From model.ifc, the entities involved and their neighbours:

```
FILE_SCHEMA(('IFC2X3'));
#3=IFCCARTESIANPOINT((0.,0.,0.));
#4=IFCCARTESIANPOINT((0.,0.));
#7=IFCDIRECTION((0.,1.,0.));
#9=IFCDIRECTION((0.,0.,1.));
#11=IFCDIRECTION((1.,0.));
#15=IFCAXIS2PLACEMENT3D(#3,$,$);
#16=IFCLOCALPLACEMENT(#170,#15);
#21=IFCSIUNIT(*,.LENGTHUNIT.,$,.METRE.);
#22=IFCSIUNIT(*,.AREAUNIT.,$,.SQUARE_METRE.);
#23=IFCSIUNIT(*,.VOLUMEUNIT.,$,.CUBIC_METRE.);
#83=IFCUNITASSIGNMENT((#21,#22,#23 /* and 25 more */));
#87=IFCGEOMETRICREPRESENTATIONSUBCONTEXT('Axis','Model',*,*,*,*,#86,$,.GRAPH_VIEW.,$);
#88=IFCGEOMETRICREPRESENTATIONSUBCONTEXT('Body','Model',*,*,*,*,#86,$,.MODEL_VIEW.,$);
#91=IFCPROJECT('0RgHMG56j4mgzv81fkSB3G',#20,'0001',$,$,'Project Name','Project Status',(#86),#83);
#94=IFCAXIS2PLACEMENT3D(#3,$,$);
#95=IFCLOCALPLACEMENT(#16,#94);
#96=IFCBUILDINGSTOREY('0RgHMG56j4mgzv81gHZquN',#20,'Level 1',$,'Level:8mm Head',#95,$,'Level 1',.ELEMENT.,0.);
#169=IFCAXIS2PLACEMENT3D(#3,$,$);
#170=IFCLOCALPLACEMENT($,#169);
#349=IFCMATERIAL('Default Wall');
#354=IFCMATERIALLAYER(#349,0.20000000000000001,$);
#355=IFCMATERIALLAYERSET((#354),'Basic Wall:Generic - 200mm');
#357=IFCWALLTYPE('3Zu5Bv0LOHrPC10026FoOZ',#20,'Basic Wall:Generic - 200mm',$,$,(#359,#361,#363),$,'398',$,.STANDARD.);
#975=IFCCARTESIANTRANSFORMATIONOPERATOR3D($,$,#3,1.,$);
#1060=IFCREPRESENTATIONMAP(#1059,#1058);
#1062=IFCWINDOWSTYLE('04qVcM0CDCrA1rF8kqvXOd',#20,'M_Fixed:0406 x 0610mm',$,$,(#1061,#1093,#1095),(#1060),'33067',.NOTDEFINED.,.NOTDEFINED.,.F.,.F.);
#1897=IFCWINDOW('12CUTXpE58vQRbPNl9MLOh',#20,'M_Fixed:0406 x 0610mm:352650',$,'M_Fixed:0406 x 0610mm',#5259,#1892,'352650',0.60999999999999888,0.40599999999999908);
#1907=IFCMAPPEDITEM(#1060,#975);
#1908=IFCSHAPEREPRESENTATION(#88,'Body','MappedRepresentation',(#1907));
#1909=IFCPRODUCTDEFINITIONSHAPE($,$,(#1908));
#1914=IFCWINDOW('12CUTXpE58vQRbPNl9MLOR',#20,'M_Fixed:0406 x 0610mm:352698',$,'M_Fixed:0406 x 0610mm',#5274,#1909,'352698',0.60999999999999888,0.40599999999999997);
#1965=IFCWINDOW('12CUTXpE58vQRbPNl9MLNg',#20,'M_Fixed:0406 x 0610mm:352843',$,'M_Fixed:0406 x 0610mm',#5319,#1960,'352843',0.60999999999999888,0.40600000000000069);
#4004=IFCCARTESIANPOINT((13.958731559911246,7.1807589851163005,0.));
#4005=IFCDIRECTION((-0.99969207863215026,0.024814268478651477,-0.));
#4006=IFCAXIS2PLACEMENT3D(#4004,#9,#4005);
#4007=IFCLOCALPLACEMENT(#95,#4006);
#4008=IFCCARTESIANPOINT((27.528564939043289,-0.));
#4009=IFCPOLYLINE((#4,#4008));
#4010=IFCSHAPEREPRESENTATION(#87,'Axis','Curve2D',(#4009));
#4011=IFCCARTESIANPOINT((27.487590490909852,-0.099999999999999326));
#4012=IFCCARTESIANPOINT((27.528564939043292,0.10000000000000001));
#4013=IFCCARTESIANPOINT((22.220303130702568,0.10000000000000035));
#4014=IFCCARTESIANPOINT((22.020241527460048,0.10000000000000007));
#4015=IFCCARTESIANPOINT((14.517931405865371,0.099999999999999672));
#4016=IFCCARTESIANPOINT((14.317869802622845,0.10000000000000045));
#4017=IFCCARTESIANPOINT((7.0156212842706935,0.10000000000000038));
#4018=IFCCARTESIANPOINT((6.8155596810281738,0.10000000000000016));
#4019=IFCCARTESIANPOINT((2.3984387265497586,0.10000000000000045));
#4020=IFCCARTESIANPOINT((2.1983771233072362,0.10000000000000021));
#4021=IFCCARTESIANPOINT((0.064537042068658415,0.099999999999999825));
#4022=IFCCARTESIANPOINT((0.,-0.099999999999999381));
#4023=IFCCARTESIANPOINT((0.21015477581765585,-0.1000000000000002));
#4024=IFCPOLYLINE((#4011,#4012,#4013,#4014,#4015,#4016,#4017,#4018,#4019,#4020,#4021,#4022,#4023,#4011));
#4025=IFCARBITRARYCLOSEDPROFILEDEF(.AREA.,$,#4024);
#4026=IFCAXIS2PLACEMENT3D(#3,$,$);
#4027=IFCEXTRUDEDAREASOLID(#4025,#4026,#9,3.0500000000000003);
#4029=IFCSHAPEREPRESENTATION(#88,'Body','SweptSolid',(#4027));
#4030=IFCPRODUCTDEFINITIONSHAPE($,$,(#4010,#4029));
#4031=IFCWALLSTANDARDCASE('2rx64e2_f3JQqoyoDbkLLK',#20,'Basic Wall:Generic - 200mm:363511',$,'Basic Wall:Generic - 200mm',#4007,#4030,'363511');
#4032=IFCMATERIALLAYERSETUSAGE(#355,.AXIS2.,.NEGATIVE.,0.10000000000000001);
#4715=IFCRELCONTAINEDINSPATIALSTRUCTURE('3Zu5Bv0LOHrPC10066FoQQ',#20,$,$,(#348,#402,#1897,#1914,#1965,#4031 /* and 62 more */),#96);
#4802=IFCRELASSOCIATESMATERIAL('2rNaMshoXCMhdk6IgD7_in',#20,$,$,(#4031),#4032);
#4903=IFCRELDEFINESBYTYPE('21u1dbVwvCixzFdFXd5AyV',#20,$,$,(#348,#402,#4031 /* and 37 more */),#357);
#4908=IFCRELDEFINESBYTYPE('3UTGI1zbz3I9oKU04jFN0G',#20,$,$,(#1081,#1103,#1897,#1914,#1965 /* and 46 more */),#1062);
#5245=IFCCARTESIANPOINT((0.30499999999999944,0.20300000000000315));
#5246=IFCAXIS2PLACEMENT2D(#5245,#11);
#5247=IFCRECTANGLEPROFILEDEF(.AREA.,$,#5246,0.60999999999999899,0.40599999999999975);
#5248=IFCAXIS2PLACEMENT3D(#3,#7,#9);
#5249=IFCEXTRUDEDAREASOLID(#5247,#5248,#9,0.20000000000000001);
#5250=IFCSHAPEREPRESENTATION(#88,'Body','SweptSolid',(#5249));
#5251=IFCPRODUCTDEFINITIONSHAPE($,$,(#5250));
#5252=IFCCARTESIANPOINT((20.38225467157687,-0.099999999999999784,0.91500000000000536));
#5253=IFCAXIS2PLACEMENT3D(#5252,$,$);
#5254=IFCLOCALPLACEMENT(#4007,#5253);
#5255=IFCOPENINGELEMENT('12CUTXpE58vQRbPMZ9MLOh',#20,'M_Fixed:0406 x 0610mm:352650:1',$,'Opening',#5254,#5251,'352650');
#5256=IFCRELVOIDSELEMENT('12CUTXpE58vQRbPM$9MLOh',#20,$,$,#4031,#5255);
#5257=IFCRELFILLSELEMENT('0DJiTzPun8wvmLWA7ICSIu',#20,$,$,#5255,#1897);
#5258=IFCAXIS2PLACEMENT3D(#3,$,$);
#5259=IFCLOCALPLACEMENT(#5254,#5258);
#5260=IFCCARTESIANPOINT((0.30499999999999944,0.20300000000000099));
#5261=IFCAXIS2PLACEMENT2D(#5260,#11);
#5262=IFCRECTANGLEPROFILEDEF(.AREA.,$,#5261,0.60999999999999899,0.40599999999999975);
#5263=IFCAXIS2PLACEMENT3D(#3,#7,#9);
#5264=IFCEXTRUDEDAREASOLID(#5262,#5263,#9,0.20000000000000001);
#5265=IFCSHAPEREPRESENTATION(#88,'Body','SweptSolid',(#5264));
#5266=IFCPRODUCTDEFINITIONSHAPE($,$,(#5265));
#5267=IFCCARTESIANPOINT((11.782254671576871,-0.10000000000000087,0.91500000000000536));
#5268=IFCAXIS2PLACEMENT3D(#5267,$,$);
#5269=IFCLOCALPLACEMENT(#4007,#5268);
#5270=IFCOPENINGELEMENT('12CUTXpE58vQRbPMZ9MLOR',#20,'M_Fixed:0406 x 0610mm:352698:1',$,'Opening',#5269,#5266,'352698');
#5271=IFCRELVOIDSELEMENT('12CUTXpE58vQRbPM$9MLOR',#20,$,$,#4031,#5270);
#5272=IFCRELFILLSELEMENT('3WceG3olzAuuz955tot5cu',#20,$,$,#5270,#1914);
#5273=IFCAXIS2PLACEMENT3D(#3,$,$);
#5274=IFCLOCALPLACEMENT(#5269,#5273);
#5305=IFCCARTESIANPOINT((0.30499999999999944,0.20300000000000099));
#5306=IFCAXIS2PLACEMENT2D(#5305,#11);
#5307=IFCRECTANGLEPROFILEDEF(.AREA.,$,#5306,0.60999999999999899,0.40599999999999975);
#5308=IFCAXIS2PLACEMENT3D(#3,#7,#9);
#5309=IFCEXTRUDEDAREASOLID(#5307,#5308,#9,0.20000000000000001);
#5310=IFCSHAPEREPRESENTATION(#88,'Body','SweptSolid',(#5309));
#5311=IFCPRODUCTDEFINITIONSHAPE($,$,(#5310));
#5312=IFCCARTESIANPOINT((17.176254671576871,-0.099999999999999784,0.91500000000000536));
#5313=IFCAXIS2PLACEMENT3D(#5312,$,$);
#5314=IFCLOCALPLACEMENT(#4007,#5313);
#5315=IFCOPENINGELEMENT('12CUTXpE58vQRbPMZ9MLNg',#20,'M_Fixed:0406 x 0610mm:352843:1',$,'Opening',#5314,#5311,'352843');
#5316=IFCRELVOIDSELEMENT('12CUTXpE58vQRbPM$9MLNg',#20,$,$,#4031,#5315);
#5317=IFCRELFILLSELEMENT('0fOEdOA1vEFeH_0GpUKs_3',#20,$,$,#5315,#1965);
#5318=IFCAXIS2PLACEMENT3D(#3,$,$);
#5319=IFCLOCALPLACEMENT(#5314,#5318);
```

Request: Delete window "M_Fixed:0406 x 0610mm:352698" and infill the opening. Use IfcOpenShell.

```python
import ifcopenshell
import ifcopenshell.api.feature
import ifcopenshell.api.root
import ifcopenshell.geom
import ifcopenshell.util.shape

model = ifcopenshell.open("model.ifc")
settings = ifcopenshell.geom.settings()


def volume(element):
    """Net volume in cubic metres, openings subtracted."""
    shape = ifcopenshell.geom.create_shape(settings, element)
    return ifcopenshell.util.shape.get_volume(shape.geometry)


window = model.by_id(1914)
opening = window.FillsVoids[0].RelatingOpeningElement
wall = opening.VoidsElements[0].RelatingBuildingElement
before = volume(wall)

ifcopenshell.api.root.remove_product(model, product=window)
ifcopenshell.api.feature.remove_feature(model, feature=opening)

after = volume(wall)

print(f"wall volume {before:.3f} -> {after:.3f} m3")

model.write("model_rev.ifc")
```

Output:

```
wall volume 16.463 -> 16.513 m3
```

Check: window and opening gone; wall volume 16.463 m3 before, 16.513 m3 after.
